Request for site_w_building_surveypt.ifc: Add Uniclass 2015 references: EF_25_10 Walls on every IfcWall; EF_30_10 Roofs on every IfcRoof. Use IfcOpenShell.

First a look at what the model holds.

```python
import ifcopenshell

model = ifcopenshell.open("site_w_building_surveypt.ifc")
print(model.schema)
print("classifications:", [c.Name for c in model.by_type("IfcClassification")])
for ifc_class in ("IfcDoor", "IfcRoof", "IfcStair", "IfcWall", "IfcWindow"):
    print(ifc_class, len(model.by_type(ifc_class)))
```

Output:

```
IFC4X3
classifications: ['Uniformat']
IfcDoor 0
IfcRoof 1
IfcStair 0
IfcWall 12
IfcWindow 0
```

```python
import ifcopenshell
import ifcopenshell.api.classification

model = ifcopenshell.open("site_w_building_surveypt.ifc")

system = ifcopenshell.api.classification.add_classification(model, classification="Uniclass 2015")

codes = {
    "IfcWall": ("EF_25_10", "Walls"),
    "IfcRoof": ("EF_30_10", "Roofs"),
}
for ifc_class, (code, name) in codes.items():
    products = model.by_type(ifc_class)
    ifcopenshell.api.classification.add_reference(
        model, products=products, classification=system, identification=code, name=name
    )
    print(code, len(products))

model.write("site_w_building_surveypt-out.ifc")
```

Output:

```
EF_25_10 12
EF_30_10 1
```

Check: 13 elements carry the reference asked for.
